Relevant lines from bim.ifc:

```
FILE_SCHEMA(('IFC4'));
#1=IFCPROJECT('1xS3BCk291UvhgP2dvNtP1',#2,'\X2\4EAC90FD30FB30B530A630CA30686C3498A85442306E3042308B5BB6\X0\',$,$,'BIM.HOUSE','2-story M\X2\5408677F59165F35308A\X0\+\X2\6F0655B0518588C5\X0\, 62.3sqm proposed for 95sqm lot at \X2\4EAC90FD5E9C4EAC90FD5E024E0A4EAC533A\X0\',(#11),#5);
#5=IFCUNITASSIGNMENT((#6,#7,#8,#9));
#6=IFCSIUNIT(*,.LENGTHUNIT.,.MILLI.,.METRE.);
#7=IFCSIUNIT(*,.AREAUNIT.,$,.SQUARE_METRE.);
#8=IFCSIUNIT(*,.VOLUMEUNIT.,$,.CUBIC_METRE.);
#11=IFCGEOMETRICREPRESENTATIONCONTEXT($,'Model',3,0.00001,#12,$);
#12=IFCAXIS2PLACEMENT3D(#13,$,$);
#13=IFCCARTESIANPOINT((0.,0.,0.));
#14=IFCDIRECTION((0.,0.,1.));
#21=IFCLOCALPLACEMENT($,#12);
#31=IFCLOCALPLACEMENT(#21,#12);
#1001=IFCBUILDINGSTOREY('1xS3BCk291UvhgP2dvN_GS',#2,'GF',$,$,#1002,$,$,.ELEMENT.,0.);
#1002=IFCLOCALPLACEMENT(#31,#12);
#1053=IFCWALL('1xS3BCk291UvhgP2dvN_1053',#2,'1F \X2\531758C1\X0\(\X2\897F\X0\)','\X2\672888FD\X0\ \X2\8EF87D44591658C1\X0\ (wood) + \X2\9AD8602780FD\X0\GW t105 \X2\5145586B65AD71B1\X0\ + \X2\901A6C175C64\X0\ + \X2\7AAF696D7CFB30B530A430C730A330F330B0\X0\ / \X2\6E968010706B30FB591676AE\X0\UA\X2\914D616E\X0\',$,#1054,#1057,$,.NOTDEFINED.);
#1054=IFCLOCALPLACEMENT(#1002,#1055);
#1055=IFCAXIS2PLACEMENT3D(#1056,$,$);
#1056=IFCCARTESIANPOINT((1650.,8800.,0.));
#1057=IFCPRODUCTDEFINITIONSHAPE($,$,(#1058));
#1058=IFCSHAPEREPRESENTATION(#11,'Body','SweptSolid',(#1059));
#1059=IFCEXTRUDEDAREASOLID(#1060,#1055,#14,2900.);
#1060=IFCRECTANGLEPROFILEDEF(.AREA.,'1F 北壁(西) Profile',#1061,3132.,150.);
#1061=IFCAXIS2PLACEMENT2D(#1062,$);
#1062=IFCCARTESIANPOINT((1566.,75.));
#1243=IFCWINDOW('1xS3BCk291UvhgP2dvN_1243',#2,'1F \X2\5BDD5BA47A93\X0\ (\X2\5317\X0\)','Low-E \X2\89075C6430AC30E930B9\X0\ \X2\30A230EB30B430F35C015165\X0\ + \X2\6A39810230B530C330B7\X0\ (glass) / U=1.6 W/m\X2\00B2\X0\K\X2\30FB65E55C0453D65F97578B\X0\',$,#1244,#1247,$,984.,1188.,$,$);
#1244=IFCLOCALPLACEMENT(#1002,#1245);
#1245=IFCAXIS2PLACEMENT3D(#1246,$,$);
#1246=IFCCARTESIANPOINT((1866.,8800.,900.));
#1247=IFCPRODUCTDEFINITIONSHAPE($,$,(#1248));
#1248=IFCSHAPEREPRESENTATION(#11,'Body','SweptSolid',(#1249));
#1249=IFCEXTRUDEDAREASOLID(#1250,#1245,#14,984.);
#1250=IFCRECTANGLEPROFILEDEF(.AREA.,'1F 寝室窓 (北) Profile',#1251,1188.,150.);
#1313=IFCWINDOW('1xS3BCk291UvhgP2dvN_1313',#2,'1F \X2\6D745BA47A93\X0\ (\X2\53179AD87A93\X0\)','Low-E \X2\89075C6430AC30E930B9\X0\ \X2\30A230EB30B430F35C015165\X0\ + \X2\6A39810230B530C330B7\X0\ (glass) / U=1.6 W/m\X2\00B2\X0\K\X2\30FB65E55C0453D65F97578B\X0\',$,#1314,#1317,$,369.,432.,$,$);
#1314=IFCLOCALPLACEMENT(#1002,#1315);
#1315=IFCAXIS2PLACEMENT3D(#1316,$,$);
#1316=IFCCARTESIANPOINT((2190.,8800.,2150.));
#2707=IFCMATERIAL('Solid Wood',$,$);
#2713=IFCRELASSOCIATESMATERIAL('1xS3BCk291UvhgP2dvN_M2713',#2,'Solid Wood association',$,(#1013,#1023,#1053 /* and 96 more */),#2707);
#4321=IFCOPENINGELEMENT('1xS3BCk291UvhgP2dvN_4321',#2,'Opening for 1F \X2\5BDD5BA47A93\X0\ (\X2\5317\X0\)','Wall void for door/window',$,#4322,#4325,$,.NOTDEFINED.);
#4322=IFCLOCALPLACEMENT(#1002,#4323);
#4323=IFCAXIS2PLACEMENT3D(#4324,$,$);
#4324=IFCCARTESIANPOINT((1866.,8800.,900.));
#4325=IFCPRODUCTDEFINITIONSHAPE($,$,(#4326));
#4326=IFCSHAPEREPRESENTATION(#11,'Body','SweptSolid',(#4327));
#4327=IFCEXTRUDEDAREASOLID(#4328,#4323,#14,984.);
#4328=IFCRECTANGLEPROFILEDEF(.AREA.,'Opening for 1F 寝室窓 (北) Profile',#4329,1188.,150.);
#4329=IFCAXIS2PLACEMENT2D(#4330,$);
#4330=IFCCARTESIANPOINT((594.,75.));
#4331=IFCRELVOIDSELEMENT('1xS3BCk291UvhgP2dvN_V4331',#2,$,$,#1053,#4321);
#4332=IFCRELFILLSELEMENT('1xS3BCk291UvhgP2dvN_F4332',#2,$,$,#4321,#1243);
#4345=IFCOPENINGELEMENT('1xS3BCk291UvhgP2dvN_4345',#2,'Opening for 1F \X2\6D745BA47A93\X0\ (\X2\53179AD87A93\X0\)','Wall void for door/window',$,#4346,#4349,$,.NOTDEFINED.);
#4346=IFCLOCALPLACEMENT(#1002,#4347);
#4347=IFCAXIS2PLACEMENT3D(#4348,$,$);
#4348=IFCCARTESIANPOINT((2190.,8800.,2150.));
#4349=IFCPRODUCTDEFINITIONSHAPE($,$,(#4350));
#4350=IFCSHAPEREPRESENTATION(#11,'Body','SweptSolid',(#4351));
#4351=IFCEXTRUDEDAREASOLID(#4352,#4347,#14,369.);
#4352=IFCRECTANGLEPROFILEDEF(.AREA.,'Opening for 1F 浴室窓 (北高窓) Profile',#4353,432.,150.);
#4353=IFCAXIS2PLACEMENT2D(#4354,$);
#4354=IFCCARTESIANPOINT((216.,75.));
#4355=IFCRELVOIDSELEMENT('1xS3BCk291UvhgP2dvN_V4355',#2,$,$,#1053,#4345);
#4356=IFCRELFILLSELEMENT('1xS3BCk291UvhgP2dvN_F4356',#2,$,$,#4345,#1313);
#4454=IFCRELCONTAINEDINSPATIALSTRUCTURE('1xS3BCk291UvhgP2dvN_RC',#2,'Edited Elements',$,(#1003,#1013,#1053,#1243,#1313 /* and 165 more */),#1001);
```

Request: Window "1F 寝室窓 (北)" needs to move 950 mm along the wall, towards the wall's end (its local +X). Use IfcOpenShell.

```python
import ifcopenshell
import ifcopenshell.api.geometry
import ifcopenshell.util.placement

model = ifcopenshell.open("bim.ifc")

window = model.by_guid("1xS3BCk291UvhgP2dvN_1243")
opening = window.FillsVoids[0].RelatingOpeningElement
wall = opening.VoidsElements[0].RelatingBuildingElement

wall_matrix = ifcopenshell.util.placement.get_local_placement(wall.ObjectPlacement)
shift = wall_matrix[:3, 0] * 950.0
before = ifcopenshell.util.placement.get_local_placement(window.ObjectPlacement)[:3, 3].copy()

# The window is not placed relative to its opening, so move both.
for product in (opening, window):
    matrix = ifcopenshell.util.placement.get_local_placement(product.ObjectPlacement)
    matrix[:3, 3] += shift
    ifcopenshell.api.geometry.edit_object_placement(model, product=product, matrix=matrix, is_si=False)

after = ifcopenshell.util.placement.get_local_placement(window.ObjectPlacement)[:3, 3]
print("window moved by", (after - before).round(3) + 0.0)

model.write("bim_updated.ifc")
```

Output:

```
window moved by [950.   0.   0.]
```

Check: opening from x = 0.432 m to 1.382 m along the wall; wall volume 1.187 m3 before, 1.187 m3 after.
